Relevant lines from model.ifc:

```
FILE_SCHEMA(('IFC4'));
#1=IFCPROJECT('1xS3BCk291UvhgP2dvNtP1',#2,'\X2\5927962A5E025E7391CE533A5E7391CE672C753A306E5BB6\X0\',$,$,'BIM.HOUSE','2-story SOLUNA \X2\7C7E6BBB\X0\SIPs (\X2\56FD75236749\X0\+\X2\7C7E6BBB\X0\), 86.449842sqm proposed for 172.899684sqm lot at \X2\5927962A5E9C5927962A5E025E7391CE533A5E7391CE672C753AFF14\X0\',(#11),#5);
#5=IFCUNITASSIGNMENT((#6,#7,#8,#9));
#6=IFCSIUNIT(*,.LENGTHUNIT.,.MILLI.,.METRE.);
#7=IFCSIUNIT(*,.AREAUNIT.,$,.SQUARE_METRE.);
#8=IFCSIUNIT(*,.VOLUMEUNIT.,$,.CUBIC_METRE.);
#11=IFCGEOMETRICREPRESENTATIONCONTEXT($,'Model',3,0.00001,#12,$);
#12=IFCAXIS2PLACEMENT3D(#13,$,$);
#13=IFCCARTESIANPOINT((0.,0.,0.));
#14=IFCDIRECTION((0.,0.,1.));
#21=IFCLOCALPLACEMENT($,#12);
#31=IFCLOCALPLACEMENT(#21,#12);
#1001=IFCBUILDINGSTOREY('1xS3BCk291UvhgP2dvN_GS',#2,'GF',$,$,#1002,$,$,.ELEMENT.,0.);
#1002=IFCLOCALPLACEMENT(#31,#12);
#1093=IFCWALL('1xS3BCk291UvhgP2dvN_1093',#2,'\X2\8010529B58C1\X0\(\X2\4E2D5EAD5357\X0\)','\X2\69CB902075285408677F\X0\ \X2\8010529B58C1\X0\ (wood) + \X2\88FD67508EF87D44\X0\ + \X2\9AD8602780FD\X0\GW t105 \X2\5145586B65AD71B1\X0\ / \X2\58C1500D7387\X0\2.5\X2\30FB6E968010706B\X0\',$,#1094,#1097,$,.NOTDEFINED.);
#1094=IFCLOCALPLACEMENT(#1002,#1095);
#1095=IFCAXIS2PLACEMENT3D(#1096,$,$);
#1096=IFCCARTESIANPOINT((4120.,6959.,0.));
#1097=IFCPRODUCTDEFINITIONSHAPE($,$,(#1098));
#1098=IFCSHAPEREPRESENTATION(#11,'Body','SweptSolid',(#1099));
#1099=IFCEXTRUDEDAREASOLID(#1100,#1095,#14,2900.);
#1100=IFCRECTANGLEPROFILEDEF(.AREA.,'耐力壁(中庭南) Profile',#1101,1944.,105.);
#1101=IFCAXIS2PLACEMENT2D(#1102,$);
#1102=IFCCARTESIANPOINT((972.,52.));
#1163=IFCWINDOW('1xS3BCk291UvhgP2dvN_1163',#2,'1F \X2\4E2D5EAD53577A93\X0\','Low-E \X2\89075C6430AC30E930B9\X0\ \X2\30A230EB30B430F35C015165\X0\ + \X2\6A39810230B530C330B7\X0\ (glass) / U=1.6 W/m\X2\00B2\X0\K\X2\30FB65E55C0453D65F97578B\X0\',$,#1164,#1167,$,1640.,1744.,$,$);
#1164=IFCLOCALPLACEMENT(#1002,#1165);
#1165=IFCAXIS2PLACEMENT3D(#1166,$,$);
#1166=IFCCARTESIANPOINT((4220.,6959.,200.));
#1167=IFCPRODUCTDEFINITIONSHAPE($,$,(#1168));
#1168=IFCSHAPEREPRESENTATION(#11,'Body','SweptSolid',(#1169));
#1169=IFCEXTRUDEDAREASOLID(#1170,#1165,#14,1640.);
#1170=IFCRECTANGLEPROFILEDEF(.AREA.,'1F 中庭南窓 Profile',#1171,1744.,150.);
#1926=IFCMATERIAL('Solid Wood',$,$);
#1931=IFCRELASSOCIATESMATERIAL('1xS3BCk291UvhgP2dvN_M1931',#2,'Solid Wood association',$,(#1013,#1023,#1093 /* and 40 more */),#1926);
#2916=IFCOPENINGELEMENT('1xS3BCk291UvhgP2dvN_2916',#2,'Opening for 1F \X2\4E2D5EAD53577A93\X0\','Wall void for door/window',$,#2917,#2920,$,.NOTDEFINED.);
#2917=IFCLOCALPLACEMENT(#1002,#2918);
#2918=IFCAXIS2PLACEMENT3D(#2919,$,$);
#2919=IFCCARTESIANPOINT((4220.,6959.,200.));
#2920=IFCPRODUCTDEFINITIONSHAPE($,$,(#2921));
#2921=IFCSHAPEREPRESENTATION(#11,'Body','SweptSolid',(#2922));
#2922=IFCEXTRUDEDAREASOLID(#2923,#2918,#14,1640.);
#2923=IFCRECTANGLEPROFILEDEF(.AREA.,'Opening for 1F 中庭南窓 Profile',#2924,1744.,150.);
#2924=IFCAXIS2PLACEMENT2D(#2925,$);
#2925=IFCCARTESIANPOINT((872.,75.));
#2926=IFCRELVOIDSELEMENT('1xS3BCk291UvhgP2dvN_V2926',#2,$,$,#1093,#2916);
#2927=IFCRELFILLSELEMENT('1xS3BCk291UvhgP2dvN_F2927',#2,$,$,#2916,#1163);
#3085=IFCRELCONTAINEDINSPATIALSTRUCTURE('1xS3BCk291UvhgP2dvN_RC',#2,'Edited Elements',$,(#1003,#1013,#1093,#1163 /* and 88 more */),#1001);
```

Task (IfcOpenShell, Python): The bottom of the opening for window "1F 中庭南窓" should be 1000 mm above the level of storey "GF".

```python
import numpy as np
import ifcopenshell
import ifcopenshell.api.geometry
import ifcopenshell.geom
import ifcopenshell.util.element
import ifcopenshell.util.placement
import ifcopenshell.util.shape
import ifcopenshell.util.unit

model = ifcopenshell.open("model.ifc")
unit_scale = ifcopenshell.util.unit.calculate_unit_scale(model)

window = model.by_id(1163)
opening = window.FillsVoids[0].RelatingOpeningElement
storey = ifcopenshell.util.element.get_container(window, ifc_class="IfcBuildingStorey")
level = ifcopenshell.util.placement.get_local_placement(storey.ObjectPlacement)[2, 3]

# The opening's origin need not be at the sill, so measure its lowest point.
shape = ifcopenshell.geom.create_shape(ifcopenshell.geom.settings(), opening)
bottom = ifcopenshell.util.shape.get_shape_bottom_elevation(shape, shape.geometry) / unit_scale
dz = level + 1 / unit_scale - bottom

shift = np.array([0.0, 0.0, dz])
# The window is not placed relative to its opening, so move both.
for product in (opening, window):
    matrix = ifcopenshell.util.placement.get_local_placement(product.ObjectPlacement)
    matrix[:3, 3] += shift
    ifcopenshell.api.geometry.edit_object_placement(model, product=product, matrix=matrix, is_si=False)

print(f"moved by {dz * unit_scale:+.3f} m")

model.write("model-out.ifc")
```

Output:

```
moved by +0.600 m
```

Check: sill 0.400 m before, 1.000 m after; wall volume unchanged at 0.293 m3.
